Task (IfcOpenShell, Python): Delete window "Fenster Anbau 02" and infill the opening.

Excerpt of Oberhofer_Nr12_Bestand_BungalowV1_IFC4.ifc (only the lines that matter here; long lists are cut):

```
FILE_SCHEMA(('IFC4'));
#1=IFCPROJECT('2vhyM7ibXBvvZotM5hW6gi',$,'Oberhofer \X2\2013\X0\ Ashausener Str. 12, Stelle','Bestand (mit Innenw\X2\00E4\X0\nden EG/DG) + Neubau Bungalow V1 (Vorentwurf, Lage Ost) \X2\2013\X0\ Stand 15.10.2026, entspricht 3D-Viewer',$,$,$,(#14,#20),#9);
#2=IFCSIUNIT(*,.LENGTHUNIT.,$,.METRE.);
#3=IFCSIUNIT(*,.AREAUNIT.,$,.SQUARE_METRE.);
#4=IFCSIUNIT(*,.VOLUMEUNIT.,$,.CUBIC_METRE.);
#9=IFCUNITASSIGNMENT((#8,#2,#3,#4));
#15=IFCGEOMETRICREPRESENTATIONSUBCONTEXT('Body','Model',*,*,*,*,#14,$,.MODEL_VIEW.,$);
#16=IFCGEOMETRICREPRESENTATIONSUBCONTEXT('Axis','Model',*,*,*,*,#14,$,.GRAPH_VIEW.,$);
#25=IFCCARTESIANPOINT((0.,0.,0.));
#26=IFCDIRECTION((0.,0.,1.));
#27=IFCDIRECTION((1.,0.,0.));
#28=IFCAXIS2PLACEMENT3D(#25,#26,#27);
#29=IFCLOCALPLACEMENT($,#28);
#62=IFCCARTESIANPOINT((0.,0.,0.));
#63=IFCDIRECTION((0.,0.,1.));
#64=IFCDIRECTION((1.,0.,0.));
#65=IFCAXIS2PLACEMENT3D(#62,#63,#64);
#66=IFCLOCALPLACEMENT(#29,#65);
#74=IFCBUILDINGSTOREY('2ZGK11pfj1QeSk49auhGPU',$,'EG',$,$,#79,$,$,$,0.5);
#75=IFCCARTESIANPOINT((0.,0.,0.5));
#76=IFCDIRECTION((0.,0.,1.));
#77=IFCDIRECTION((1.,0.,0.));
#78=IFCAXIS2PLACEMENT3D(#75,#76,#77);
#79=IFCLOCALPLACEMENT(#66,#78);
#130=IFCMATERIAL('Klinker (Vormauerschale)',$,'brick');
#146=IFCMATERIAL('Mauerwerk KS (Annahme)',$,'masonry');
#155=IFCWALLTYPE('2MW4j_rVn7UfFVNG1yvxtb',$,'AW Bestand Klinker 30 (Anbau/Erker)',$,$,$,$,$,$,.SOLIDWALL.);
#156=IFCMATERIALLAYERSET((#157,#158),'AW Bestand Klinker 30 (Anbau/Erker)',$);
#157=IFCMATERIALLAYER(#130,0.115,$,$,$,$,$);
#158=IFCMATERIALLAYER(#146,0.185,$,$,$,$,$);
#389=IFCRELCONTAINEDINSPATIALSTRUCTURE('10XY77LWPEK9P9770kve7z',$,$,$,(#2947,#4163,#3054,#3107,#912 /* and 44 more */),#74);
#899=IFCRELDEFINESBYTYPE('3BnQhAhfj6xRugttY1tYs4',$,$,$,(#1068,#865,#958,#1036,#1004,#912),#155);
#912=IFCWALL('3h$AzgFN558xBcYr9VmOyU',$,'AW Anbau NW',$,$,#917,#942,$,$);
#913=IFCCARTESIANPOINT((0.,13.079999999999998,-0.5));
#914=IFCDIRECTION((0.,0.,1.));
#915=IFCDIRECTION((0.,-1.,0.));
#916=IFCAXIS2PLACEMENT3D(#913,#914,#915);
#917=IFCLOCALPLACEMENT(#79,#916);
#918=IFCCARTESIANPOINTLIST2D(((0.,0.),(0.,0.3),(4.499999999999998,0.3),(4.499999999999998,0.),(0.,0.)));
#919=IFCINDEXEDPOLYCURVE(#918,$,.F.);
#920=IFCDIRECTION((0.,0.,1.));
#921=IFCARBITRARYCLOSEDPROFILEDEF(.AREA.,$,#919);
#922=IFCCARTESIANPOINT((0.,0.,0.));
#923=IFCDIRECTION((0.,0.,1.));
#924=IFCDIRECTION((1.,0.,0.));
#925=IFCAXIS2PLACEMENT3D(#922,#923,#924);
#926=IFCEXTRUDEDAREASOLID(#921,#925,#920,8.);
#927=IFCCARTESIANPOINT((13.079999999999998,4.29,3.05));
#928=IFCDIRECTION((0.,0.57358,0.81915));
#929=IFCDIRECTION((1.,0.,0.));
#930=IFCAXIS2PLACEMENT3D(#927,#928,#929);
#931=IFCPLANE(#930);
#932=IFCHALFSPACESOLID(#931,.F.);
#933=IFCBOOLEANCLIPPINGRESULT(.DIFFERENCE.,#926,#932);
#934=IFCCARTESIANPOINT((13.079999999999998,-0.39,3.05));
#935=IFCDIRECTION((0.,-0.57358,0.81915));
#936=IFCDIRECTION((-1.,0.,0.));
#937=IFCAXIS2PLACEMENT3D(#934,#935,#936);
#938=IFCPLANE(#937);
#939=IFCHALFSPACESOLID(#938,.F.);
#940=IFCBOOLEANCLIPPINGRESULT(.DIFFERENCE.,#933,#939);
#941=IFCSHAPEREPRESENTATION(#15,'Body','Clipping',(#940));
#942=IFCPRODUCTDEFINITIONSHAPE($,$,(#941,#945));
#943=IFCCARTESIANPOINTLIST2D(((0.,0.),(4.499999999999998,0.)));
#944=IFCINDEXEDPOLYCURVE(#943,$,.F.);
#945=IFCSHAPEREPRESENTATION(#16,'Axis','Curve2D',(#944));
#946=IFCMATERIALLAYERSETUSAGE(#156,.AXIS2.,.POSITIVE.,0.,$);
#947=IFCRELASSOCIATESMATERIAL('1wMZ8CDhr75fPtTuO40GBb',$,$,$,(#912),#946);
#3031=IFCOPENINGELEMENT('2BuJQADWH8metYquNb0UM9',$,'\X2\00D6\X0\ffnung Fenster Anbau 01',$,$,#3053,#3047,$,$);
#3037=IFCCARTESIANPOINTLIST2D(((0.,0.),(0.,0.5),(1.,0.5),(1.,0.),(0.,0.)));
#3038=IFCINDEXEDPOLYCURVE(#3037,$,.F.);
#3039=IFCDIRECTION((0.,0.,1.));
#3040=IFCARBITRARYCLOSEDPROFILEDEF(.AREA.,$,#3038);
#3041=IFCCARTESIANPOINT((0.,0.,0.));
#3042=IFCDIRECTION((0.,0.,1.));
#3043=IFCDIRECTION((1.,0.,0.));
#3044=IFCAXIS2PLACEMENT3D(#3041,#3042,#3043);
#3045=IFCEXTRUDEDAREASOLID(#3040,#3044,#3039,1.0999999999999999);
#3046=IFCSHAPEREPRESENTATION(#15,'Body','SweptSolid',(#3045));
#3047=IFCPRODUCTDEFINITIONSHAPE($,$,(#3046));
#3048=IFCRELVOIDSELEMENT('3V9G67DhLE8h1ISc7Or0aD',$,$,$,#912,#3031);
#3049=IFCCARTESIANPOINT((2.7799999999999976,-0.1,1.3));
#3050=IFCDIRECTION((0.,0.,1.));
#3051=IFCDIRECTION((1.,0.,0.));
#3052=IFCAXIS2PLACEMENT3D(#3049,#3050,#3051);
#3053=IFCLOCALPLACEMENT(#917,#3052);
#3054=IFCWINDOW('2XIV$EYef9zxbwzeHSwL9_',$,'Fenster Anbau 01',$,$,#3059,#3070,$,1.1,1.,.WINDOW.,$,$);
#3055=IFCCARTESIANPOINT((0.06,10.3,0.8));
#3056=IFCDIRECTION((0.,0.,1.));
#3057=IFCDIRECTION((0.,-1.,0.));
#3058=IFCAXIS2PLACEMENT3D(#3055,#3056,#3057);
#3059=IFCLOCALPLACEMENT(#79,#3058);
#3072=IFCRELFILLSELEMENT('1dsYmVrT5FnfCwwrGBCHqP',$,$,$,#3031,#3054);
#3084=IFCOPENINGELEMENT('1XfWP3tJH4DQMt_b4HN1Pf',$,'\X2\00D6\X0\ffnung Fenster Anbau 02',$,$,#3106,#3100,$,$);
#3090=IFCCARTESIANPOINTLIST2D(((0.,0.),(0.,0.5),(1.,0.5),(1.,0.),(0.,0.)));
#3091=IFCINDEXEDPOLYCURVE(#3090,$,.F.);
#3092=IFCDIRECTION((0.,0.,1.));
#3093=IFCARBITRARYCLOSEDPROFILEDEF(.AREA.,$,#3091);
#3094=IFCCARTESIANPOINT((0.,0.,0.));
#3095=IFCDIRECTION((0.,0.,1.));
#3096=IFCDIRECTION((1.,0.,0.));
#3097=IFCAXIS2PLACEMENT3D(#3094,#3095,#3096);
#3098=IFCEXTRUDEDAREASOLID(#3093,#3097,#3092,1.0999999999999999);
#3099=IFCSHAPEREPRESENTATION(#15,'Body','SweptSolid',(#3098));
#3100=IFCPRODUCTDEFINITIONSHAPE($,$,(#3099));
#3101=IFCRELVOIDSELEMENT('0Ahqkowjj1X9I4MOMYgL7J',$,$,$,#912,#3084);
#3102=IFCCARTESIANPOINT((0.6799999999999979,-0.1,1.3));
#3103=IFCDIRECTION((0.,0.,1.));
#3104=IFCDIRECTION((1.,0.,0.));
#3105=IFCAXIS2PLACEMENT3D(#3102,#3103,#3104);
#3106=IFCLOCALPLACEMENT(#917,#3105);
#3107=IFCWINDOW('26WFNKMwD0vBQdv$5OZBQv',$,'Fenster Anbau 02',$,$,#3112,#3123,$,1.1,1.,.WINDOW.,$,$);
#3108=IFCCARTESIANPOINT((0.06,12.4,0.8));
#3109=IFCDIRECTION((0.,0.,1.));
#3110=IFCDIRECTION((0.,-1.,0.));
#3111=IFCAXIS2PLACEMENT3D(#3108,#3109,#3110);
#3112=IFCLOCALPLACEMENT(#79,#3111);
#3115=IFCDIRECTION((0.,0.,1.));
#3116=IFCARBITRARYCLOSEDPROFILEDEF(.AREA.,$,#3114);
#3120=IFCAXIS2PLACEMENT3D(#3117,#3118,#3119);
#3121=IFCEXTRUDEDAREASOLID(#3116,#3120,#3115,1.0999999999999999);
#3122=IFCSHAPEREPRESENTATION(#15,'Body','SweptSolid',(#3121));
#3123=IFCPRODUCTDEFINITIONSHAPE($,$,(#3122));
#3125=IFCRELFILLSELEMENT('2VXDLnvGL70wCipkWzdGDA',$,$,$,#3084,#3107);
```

```python
import ifcopenshell
import ifcopenshell.api.feature
import ifcopenshell.api.root
import ifcopenshell.geom
import ifcopenshell.util.shape

model = ifcopenshell.open("Oberhofer_Nr12_Bestand_BungalowV1_IFC4.ifc")
settings = ifcopenshell.geom.settings()


def volume(element):
    """Net volume in cubic metres, openings subtracted."""
    shape = ifcopenshell.geom.create_shape(settings, element)
    return ifcopenshell.util.shape.get_volume(shape.geometry)


window = model.by_guid("26WFNKMwD0vBQdv$5OZBQv")
opening = window.FillsVoids[0].RelatingOpeningElement
wall = opening.VoidsElements[0].RelatingBuildingElement
before = volume(wall)

ifcopenshell.api.root.remove_product(model, product=window)
ifcopenshell.api.feature.remove_feature(model, feature=opening)

after = volume(wall)

print(f"wall volume {before:.3f} -> {after:.3f} m3")

model.write("Oberhofer_Nr12_Bestand_BungalowV1_IFC4_edited.ifc")
```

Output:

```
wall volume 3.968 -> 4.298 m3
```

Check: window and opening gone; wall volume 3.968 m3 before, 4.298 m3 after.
